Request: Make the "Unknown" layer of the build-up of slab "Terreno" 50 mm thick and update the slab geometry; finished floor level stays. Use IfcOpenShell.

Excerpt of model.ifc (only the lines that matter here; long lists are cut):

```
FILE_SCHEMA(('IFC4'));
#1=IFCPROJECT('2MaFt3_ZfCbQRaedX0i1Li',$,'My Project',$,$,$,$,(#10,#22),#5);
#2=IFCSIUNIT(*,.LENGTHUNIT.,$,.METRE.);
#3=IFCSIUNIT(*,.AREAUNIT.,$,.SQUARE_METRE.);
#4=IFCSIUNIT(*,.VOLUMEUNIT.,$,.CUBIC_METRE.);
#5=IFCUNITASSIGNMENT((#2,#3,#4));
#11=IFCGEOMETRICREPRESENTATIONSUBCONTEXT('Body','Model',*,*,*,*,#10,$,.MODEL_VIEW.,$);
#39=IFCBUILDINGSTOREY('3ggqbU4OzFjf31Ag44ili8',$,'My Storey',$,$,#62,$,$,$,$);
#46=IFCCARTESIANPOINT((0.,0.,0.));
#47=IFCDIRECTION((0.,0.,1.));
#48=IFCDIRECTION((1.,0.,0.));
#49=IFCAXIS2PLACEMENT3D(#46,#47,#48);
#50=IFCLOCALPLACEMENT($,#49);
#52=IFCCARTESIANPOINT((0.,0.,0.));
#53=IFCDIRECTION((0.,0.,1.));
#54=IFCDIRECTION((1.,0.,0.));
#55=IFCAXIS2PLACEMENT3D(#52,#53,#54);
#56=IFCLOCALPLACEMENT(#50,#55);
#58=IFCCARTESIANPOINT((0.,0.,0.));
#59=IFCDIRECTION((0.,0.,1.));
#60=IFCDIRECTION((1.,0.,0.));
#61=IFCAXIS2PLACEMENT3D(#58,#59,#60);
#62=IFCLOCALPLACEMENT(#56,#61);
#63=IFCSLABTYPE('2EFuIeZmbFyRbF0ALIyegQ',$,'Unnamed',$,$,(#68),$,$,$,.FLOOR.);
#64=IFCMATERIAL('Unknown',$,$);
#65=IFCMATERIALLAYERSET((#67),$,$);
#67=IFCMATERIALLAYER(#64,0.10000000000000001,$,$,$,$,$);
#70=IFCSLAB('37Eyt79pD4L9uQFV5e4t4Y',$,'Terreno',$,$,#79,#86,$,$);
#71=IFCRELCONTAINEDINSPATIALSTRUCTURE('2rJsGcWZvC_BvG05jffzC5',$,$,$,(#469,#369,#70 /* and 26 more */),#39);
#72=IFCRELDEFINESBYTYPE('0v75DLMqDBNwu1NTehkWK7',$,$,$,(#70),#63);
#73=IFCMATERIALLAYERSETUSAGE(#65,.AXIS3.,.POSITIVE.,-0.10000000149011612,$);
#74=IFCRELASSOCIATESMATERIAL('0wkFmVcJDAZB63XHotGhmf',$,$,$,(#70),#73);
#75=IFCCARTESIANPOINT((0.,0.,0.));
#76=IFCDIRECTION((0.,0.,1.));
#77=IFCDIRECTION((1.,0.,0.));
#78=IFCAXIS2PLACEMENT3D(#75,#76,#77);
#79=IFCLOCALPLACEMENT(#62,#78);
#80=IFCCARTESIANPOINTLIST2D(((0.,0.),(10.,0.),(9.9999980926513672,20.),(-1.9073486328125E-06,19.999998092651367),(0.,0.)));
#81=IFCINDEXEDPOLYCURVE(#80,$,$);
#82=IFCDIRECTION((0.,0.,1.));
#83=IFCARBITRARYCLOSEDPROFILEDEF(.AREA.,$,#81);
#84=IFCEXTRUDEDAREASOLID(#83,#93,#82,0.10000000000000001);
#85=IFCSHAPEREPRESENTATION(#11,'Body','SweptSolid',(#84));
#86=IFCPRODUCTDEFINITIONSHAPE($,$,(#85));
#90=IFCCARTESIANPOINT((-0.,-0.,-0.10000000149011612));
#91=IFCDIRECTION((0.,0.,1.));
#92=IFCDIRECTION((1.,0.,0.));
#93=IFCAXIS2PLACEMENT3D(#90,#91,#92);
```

```python
import ifcopenshell
import ifcopenshell.util.element
import ifcopenshell.util.representation

model = ifcopenshell.open("model.ifc")

layer_set = model.by_id(65)
layer = next(l for l in layer_set.MaterialLayers if l.Material and l.Material.Name == "Unknown")
change = 0.05 - layer.LayerThickness
layer.LayerThickness += change

# Geometry does not follow the layer set by itself.
slabs = [e for e in ifcopenshell.util.element.get_elements_by_material(model, layer_set) if e.is_a("IfcSlab")]
for slab in sorted(slabs, key=lambda e: e.id()):
    body = ifcopenshell.util.representation.get_representation(slab, "Model", "Body")
    solid = body.Items[0]
    old_depth = solid.Depth
    solid.Depth += change
    # Extruded upwards: lower the start of the extrusion so the top stays.
    x, y, z = solid.Position.Location.Coordinates
    solid.Position.Location = model.createIfcCartesianPoint((x, y, z - change))
    print(slab.id(), f"{old_depth:g} -> {solid.Depth:g}")

# The layers are counted up from the underside, which has moved.
for usage in {ifcopenshell.util.element.get_material(slab) for slab in slabs}:
    usage.OffsetFromReferenceLine -= change

model.write("model_v2.ifc")
```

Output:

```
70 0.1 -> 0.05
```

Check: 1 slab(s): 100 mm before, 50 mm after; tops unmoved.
